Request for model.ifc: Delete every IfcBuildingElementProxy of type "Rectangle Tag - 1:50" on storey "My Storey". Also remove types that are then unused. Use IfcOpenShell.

First a look at what the model holds.

```python
import ifcopenshell
import ifcopenshell.util.element

model = ifcopenshell.open("model.ifc")
print(model.schema)
storey = next(s for s in model.by_type("IfcBuildingStorey") if s.Name == "My Storey")
proxies = [e for e in ifcopenshell.util.element.get_decomposition(storey) if e.is_a("IfcBuildingElementProxy")]
seen = {}
for e in proxies:
    element_type = ifcopenshell.util.element.get_type(e)
    name = element_type.Name if element_type not in (None, e) else None
    seen[name] = seen.get(name, 0) + 1
for name, count in sorted(seen.items(), key=str):
    print(count, "x", name)
```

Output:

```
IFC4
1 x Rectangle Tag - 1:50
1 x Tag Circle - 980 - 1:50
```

```python
import ifcopenshell
import ifcopenshell.api.root
import ifcopenshell.util.element

model = ifcopenshell.open("model.ifc")

storey = next(s for s in model.by_type("IfcBuildingStorey") if s.Name == "My Storey")
proxies = [e for e in ifcopenshell.util.element.get_decomposition(storey) if e.is_a("IfcBuildingElementProxy")]
targets = [e for e in proxies if (t := ifcopenshell.util.element.get_type(e)) not in (None, e) and t.Name == "Rectangle Tag - 1:50"]
types = {ifcopenshell.util.element.get_type(e) for e in targets} - {None, *targets}

for e in targets:
    ifcopenshell.api.root.remove_product(model, product=e)
print(len(targets), "removed")

unused = [t for t in types if not ifcopenshell.util.element.get_types(t)]
for t in unused:
    ifcopenshell.api.root.remove_product(model, product=t)
print(len(unused), "unused types removed")

model.write("model_edited.ifc")
```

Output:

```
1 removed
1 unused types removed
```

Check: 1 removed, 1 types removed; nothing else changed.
